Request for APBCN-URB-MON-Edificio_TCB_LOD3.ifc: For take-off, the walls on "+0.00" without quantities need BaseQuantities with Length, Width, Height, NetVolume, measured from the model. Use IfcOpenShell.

First a look at what the model holds.

```python
import ifcopenshell
import ifcopenshell.util.element
import ifcopenshell.util.unit

model = ifcopenshell.open("APBCN-URB-MON-Edificio_TCB_LOD3.ifc")
print(model.schema)
for unit_type in ("LENGTHUNIT", "AREAUNIT", "VOLUMEUNIT"):
    print(unit_type, ifcopenshell.util.unit.calculate_unit_scale(model, unit_type))
storey = next(s for s in model.by_type("IfcBuildingStorey") if s.Name == "+0.00")
walls = [e for e in ifcopenshell.util.element.get_decomposition(storey) if e.is_a("IfcWall")]
for e in sorted(walls, key=lambda e: e.id()):
    print(e.id(), e.is_a(), e.Name, list(ifcopenshell.util.element.get_psets(e, qtos_only=True)), sep=" | ")
```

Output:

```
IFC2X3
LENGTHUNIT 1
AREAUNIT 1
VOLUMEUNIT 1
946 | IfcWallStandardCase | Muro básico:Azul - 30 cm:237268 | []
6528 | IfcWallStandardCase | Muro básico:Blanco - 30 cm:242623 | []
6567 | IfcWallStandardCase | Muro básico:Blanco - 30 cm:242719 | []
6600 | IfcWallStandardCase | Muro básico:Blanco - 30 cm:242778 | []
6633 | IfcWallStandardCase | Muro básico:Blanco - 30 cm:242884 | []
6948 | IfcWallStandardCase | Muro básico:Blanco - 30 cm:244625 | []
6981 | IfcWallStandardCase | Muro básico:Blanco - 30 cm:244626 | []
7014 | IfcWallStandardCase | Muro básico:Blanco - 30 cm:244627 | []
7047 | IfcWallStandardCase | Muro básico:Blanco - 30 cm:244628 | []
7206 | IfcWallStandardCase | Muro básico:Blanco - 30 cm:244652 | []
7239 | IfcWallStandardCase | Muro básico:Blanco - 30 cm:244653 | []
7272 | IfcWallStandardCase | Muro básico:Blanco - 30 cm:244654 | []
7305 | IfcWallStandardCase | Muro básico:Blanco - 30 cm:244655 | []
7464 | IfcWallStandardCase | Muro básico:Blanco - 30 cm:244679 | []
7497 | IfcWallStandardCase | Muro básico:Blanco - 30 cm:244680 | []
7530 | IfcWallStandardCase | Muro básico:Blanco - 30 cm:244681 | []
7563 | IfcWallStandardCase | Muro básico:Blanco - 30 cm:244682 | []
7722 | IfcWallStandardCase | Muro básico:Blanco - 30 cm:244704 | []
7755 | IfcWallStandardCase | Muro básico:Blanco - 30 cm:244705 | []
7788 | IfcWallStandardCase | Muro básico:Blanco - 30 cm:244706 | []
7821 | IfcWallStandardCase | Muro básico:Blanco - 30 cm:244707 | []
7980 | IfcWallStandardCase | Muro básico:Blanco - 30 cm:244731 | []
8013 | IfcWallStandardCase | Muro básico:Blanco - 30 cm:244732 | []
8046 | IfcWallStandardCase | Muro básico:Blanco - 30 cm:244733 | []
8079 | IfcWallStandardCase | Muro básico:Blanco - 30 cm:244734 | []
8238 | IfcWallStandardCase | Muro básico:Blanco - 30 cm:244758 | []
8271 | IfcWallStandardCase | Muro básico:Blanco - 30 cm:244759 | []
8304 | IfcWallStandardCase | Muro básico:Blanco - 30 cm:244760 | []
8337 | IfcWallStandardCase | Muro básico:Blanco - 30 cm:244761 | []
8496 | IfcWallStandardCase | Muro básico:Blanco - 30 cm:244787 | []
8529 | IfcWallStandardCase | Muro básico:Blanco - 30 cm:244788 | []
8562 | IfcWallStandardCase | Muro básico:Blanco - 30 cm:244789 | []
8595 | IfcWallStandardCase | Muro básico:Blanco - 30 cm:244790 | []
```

```python
import ifcopenshell
import ifcopenshell.api.pset
import ifcopenshell.geom
import ifcopenshell.util.element
import ifcopenshell.util.shape
import ifcopenshell.util.unit

model = ifcopenshell.open("APBCN-URB-MON-Edificio_TCB_LOD3.ifc")
unit_scale = ifcopenshell.util.unit.calculate_unit_scale(model)
volume_scale = ifcopenshell.util.unit.calculate_unit_scale(model, "VOLUMEUNIT")
settings = ifcopenshell.geom.settings()

storey = next(s for s in model.by_type("IfcBuildingStorey") if s.Name == "+0.00")
walls = [e for e in ifcopenshell.util.element.get_decomposition(storey) if e.is_a("IfcWall")]

for e in sorted(walls, key=lambda e: e.id()):
    if ifcopenshell.util.element.get_psets(e, qtos_only=True, should_inherit=False):
        continue
    # Geometry comes back in metres, in the element's own axes.
    shape = ifcopenshell.geom.create_shape(settings, e)
    values = {
        "Length": ifcopenshell.util.shape.get_x(shape.geometry) / unit_scale,
        "Width": ifcopenshell.util.shape.get_y(shape.geometry) / unit_scale,
        "Height": ifcopenshell.util.shape.get_z(shape.geometry) / unit_scale,
        "NetVolume": ifcopenshell.util.shape.get_volume(shape.geometry) / volume_scale,
    }
    qto = ifcopenshell.api.pset.add_qto(model, product=e, name="BaseQuantities")
    ifcopenshell.api.pset.edit_qto(model, qto=qto, properties=values)
    print(e.id(), {k: round(v, 3) for k, v in values.items()})

model.write("APBCN-URB-MON-Edificio_TCB_LOD3_edited.ifc")
```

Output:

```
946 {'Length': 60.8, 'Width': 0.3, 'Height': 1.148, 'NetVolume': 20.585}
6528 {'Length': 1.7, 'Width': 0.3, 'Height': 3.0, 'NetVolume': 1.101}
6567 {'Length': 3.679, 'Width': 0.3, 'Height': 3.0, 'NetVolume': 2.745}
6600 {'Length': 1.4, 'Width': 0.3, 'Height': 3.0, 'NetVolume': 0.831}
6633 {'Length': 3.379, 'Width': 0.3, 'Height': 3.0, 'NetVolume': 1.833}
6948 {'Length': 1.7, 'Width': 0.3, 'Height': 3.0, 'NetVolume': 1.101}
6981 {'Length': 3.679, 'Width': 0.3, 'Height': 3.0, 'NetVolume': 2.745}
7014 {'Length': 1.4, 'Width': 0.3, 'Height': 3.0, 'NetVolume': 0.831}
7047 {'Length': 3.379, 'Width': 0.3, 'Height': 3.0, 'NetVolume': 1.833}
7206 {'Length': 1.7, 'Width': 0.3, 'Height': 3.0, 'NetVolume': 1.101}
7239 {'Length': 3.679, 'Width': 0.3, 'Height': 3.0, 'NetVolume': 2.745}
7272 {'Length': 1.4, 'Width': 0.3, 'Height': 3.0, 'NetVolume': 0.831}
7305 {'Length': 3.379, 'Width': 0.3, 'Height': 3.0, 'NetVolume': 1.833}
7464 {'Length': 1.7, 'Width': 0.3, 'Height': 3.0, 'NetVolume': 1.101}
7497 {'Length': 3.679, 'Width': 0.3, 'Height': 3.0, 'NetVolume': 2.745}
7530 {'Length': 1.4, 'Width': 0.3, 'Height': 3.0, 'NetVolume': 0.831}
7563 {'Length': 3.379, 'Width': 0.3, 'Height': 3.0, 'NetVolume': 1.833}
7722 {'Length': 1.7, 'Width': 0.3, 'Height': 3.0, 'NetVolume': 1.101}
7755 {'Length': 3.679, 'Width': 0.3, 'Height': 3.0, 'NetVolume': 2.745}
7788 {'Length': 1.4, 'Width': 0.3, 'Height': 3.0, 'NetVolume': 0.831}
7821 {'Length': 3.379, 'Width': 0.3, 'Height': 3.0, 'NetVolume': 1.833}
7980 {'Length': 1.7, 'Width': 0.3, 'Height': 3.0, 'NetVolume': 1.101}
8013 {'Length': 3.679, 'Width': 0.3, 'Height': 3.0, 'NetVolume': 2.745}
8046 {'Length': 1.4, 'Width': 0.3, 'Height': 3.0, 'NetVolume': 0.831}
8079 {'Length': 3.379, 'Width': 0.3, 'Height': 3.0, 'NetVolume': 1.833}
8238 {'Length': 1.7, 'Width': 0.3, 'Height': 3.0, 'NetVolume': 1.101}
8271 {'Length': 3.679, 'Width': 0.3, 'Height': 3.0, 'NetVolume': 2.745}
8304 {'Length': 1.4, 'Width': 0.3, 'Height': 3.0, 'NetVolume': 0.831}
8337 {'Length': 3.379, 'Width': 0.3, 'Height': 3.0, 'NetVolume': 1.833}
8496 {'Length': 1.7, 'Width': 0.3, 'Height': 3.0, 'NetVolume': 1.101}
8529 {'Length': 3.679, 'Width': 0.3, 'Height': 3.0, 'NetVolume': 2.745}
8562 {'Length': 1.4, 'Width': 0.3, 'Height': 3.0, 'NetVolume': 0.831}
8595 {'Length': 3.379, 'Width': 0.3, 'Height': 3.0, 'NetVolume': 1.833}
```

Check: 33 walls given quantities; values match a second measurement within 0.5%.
